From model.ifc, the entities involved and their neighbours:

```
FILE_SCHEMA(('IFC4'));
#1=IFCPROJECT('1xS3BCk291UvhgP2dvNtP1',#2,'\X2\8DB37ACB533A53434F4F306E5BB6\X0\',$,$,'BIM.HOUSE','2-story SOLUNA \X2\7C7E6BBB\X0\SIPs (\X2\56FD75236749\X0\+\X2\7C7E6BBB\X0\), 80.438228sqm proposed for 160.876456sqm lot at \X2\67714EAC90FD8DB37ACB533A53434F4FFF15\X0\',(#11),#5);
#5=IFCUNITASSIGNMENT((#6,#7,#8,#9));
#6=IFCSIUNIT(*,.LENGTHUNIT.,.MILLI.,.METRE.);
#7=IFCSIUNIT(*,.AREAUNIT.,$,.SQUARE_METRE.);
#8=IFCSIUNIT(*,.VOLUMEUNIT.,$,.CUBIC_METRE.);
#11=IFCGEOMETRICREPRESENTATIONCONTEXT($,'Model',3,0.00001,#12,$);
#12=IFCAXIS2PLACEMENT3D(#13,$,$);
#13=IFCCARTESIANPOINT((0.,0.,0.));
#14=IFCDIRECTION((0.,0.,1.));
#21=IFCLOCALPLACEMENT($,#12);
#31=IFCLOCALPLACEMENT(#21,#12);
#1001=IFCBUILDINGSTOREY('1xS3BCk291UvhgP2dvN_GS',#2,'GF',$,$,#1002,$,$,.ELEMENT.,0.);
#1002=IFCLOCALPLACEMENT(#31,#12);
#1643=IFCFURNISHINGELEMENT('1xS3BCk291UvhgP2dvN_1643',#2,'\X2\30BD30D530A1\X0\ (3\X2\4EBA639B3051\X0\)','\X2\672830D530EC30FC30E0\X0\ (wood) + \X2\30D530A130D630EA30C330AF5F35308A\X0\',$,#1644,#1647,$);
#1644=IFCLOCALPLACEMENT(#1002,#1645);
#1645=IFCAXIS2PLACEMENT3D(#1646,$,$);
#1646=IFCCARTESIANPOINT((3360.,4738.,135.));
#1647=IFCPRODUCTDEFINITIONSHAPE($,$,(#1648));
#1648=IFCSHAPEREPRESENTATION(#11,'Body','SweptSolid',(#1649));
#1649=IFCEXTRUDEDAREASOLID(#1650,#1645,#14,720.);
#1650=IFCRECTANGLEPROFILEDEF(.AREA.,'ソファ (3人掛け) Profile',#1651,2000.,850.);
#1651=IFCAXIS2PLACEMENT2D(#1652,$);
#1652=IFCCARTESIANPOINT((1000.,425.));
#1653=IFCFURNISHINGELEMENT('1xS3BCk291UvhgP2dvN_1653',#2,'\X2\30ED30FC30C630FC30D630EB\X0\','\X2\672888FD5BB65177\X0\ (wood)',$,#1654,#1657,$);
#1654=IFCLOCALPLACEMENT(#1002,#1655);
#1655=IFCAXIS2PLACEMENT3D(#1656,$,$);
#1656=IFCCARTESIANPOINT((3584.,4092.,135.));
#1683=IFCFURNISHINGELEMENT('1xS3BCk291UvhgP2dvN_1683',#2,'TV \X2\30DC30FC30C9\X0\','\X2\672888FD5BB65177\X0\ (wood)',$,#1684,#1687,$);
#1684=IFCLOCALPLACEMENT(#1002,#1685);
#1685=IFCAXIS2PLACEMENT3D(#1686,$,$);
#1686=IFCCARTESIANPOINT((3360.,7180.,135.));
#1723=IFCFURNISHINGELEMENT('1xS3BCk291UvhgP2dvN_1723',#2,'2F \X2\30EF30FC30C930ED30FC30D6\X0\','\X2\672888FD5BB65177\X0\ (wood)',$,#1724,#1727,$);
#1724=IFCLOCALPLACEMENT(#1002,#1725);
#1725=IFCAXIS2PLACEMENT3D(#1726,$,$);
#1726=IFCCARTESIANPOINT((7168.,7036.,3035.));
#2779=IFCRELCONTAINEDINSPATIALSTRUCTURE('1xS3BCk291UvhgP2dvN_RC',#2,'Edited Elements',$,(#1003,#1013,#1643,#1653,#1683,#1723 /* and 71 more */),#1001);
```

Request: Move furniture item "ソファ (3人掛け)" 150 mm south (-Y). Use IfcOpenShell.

```python
import ifcopenshell
import ifcopenshell.api.geometry
import ifcopenshell.util.placement

model = ifcopenshell.open("model.ifc")

item = model.by_guid("1xS3BCk291UvhgP2dvN_1643")
matrix = ifcopenshell.util.placement.get_local_placement(item.ObjectPlacement)
matrix[1, 3] -= 150.0
ifcopenshell.api.geometry.edit_object_placement(model, product=item, matrix=matrix, is_si=False)

print(ifcopenshell.util.placement.get_local_placement(item.ObjectPlacement).round(3) + 0.0)

model.write("model_rev.ifc")
```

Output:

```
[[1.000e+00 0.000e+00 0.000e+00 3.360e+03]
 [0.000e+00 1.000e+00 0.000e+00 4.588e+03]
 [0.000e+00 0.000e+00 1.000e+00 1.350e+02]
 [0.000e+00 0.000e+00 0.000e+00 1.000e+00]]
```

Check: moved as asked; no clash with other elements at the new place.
